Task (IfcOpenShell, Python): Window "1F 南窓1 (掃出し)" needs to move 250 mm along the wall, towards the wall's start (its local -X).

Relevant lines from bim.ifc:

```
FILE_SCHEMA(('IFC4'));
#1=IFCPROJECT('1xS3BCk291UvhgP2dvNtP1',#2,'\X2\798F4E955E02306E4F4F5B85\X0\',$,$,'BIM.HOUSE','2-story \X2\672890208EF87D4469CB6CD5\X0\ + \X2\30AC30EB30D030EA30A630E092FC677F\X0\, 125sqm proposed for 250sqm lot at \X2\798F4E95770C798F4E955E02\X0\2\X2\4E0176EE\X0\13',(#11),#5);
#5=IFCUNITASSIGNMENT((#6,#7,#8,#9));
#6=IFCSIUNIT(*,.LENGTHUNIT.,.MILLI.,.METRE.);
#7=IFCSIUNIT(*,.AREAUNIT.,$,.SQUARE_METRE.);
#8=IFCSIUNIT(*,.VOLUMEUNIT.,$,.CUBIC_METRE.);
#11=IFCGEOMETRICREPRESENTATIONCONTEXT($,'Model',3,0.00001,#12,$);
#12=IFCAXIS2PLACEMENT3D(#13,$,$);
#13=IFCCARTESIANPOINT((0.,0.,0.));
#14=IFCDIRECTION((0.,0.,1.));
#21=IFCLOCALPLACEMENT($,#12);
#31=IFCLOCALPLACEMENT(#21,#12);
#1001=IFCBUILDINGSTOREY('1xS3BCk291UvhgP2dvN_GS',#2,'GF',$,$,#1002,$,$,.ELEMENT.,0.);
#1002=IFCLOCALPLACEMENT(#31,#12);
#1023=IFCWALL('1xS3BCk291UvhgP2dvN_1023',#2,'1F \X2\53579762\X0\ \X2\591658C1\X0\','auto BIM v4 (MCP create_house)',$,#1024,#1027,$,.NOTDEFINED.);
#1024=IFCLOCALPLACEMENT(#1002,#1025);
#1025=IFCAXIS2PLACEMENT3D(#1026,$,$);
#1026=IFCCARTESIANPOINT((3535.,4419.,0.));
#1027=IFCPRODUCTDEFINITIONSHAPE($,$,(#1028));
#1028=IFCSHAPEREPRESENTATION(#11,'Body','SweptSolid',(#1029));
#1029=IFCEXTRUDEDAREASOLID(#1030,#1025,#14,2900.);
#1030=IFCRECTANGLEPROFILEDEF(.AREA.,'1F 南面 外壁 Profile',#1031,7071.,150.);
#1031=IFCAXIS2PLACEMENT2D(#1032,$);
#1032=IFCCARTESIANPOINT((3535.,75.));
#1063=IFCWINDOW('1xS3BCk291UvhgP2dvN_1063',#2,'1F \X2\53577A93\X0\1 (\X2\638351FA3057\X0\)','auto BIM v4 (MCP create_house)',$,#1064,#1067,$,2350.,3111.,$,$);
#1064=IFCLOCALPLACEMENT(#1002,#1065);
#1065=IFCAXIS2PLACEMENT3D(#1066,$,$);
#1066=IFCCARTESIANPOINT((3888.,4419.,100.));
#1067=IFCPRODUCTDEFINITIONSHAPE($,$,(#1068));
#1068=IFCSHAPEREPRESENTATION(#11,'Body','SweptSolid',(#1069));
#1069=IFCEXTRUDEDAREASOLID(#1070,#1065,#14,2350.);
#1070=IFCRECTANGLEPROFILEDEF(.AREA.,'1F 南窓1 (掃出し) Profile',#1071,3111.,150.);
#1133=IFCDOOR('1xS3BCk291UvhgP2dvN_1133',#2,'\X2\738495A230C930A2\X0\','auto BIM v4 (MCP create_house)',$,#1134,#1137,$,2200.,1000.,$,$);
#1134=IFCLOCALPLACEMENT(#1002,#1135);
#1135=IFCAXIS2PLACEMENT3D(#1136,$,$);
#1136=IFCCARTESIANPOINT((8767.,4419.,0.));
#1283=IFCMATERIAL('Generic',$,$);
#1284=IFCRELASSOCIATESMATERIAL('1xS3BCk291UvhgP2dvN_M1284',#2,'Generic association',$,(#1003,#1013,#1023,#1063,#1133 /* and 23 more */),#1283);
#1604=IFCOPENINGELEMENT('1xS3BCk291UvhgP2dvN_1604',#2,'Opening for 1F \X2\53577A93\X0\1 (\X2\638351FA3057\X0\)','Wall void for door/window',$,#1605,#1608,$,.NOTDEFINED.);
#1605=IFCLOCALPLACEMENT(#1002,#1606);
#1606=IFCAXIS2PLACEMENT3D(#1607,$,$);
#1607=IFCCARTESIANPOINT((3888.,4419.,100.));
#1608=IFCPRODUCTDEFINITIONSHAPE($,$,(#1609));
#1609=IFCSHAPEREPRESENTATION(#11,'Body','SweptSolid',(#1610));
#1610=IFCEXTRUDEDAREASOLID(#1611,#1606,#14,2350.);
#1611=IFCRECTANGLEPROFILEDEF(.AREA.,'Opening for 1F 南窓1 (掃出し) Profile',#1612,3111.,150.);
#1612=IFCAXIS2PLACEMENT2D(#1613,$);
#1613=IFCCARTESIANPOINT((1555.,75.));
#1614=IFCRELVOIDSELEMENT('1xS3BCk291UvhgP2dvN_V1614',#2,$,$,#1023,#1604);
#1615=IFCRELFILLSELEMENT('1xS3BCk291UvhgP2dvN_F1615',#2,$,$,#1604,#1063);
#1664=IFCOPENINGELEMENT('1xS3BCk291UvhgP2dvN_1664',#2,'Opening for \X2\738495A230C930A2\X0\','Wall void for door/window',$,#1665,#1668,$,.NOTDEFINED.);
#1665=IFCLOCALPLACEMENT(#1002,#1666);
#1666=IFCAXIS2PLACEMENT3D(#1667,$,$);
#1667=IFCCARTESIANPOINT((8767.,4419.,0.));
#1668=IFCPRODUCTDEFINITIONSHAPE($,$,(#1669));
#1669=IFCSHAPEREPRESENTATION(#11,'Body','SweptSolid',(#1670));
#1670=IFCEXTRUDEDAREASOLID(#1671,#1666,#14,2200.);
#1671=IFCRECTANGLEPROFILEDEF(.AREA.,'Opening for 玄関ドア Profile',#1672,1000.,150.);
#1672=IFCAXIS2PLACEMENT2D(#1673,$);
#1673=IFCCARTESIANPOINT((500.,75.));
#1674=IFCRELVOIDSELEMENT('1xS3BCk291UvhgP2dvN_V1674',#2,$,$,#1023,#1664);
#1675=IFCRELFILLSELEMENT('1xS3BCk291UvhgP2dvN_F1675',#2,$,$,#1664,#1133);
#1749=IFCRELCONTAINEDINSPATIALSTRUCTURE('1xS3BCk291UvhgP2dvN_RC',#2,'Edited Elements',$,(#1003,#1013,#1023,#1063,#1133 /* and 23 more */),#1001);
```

```python
import ifcopenshell
import ifcopenshell.api.geometry
import ifcopenshell.util.placement
import ifcopenshell.util.unit

model = ifcopenshell.open("bim.ifc")
unit_scale = ifcopenshell.util.unit.calculate_unit_scale(model)

window = model.by_guid("1xS3BCk291UvhgP2dvN_1063")
opening = window.FillsVoids[0].RelatingOpeningElement
wall = opening.VoidsElements[0].RelatingBuildingElement

wall_matrix = ifcopenshell.util.placement.get_local_placement(wall.ObjectPlacement)
shift = wall_matrix[:3, 0] * -0.25 / unit_scale
before = ifcopenshell.util.placement.get_local_placement(window.ObjectPlacement)[:3, 3].copy()

# The window is not placed relative to its opening, so move both.
for product in (opening, window):
    matrix = ifcopenshell.util.placement.get_local_placement(product.ObjectPlacement)
    matrix[:3, 3] += shift
    ifcopenshell.api.geometry.edit_object_placement(model, product=product, matrix=matrix, is_si=False)

after = ifcopenshell.util.placement.get_local_placement(window.ObjectPlacement)[:3, 3]
print("window moved by", (after - before).round(3) + 0.0)

model.write("bim_v2.ifc")
```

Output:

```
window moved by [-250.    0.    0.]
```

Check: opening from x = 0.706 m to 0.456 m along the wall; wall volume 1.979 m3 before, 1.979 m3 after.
